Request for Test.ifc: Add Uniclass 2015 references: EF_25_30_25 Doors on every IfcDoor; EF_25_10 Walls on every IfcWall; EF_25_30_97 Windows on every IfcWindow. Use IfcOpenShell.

First a look at what the model holds.

```python
import ifcopenshell

model = ifcopenshell.open("Test.ifc")
print(model.schema)
print("classifications:", [c.Name for c in model.by_type("IfcClassification")])
for ifc_class in ("IfcDoor", "IfcRoof", "IfcStair", "IfcWall", "IfcWindow"):
    print(ifc_class, len(model.by_type(ifc_class)))
```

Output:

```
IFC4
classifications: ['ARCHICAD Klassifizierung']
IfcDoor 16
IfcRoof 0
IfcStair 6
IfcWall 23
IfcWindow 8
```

```python
import ifcopenshell
import ifcopenshell.api.classification

model = ifcopenshell.open("Test.ifc")

system = ifcopenshell.api.classification.add_classification(model, classification="Uniclass 2015")

codes = {
    "IfcDoor": ("EF_25_30_25", "Doors"),
    "IfcWall": ("EF_25_10", "Walls"),
    "IfcWindow": ("EF_25_30_97", "Windows"),
}
for ifc_class, (code, name) in codes.items():
    products = model.by_type(ifc_class)
    ifcopenshell.api.classification.add_reference(
        model, products=products, classification=system, identification=code, name=name
    )
    print(code, len(products))

model.write("Test_rev.ifc")
```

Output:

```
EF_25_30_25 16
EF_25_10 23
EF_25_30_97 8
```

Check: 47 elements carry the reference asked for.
